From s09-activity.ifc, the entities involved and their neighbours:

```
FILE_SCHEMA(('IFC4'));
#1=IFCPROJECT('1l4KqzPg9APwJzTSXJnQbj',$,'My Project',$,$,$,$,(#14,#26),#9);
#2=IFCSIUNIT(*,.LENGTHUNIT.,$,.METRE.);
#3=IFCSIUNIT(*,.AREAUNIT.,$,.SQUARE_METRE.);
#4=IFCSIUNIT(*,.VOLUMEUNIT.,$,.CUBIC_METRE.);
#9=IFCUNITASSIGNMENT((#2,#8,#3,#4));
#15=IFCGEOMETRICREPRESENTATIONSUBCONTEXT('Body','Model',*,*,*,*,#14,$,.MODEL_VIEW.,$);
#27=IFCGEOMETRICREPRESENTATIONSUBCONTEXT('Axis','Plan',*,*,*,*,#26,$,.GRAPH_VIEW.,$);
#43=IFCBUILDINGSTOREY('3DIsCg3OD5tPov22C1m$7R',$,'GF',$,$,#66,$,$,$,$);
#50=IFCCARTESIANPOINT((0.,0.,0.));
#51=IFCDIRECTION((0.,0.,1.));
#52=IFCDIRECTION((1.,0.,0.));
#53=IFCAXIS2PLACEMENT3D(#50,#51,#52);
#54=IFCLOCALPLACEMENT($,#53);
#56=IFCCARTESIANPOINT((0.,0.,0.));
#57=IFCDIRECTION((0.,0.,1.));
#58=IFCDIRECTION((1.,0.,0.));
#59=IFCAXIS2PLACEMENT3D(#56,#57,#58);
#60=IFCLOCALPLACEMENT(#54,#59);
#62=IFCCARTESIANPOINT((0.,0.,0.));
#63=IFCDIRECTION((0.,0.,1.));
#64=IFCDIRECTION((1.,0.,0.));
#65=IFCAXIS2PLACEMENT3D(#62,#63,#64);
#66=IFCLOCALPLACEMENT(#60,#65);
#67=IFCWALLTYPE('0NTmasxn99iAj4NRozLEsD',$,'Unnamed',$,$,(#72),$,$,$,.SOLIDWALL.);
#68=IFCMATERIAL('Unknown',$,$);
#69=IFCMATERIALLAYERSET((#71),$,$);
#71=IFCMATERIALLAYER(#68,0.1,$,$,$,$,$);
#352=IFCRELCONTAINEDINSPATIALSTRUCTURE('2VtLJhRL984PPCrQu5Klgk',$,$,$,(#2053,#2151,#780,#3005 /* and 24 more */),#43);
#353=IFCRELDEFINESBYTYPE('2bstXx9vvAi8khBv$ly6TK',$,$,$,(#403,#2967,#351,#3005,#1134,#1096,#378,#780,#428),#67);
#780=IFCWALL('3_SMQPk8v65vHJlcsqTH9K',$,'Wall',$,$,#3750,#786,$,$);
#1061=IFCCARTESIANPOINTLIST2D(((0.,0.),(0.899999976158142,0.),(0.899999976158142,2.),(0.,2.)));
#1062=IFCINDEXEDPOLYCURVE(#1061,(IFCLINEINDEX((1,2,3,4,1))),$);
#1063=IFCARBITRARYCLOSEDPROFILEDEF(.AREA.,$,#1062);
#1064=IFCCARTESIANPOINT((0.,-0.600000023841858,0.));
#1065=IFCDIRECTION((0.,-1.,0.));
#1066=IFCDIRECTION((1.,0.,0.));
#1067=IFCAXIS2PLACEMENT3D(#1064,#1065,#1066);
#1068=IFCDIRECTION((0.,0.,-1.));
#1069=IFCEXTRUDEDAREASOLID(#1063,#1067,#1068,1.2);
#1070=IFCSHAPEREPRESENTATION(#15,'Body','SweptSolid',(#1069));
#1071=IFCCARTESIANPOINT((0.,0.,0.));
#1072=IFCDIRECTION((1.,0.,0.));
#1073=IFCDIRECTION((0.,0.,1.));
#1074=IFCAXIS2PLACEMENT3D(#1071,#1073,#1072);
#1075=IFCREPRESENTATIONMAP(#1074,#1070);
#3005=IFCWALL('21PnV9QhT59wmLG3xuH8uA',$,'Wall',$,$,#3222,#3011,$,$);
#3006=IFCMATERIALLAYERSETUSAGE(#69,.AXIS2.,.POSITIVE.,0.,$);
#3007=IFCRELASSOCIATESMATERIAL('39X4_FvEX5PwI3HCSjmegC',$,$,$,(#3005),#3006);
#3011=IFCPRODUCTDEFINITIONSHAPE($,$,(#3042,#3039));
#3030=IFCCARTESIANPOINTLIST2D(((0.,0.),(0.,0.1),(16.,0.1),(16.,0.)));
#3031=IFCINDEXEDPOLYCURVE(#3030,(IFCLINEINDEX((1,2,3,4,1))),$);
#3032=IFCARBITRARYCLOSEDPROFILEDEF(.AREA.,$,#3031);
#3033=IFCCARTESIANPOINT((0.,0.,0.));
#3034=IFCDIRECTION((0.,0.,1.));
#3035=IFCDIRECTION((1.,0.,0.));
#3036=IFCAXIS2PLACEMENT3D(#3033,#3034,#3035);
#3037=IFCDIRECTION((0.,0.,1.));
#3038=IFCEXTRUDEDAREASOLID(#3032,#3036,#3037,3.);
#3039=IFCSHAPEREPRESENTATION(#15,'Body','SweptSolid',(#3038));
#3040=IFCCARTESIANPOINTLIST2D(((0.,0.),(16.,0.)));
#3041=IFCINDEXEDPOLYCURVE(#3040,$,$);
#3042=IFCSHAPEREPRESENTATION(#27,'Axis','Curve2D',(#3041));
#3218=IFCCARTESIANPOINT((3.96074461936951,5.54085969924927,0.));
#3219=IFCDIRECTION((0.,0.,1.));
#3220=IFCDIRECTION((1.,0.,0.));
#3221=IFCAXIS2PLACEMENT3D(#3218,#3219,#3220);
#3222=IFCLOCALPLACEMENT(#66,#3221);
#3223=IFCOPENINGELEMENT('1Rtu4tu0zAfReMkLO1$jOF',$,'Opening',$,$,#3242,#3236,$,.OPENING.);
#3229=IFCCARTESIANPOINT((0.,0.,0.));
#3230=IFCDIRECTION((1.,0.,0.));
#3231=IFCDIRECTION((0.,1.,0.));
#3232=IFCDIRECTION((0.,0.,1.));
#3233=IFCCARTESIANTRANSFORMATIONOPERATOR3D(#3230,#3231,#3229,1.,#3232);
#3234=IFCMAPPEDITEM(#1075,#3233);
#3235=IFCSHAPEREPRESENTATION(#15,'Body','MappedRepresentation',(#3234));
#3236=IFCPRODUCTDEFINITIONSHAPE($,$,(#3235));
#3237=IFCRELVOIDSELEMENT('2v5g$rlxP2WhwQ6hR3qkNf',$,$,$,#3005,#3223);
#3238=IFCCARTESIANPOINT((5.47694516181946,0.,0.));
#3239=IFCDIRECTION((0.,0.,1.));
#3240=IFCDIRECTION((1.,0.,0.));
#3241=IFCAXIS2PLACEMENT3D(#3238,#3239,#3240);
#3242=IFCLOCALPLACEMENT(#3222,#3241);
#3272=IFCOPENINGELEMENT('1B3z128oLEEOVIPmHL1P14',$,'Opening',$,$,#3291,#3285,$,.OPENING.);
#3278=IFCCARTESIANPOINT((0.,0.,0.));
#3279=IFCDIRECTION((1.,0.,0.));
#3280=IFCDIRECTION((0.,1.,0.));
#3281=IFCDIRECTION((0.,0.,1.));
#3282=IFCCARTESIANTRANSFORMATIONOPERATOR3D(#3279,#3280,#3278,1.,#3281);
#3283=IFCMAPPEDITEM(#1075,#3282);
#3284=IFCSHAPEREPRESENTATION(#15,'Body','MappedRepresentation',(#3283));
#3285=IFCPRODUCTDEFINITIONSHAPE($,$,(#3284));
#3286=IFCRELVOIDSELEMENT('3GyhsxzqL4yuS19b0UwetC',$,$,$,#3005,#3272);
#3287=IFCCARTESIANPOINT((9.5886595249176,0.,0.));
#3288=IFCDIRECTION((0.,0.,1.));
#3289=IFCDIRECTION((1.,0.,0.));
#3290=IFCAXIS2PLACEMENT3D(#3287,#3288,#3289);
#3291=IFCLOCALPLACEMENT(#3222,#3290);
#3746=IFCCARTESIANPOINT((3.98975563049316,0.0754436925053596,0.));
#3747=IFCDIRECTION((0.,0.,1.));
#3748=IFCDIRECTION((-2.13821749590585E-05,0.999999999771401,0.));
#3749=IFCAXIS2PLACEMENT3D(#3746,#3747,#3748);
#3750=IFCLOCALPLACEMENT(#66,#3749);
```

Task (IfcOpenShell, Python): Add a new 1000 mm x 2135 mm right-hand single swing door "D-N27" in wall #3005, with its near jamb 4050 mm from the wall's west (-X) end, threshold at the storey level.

```python
import numpy as np
import ifcopenshell
import ifcopenshell.api.feature
import ifcopenshell.api.geometry
import ifcopenshell.api.root
import ifcopenshell.api.spatial
import ifcopenshell.geom
import ifcopenshell.util.element
import ifcopenshell.util.placement
import ifcopenshell.util.representation
import ifcopenshell.util.shape
import ifcopenshell.util.unit

model = ifcopenshell.open("s09-activity.ifc")
unit_scale = ifcopenshell.util.unit.calculate_unit_scale(model)
settings = ifcopenshell.geom.settings()


def volume(element):
    """Net volume in cubic metres, openings subtracted."""
    shape = ifcopenshell.geom.create_shape(settings, element)
    return ifcopenshell.util.shape.get_volume(shape.geometry)


wall = model.by_guid("21PnV9QhT59wmLG3xuH8uA")
storey = ifcopenshell.util.element.get_container(wall, ifc_class="IfcBuildingStorey")
context = ifcopenshell.util.representation.get_context(model, "Model", "Body", "MODEL_VIEW")
before = volume(wall)

width, height, from_end, sill = 1, 2.135, 4.05, 0.0  # metres

# The wall runs along its own X axis, and the end named is its -X end.
wall_shape = ifcopenshell.geom.create_shape(settings, wall)
x, y, z = ifcopenshell.util.shape.get_vertices(wall_shape.geometry).T
start = x.min() + from_end
face, thickness = float(y.min()), float(y.max() - y.min())
wall_matrix = ifcopenshell.util.placement.get_local_placement(wall.ObjectPlacement)
level = ifcopenshell.util.placement.get_local_placement(storey.ObjectPlacement)[2, 3]


def in_wall(x, y):
    """Placement at x, y metres in the wall's axes, at sill height."""
    matrix = wall_matrix.copy()
    matrix[:, 3] = wall_matrix @ np.array([x / unit_scale, y / unit_scale, 0.0, 1.0])
    matrix[2, 3] = level + sill / unit_scale
    return matrix


# Opening: a box that overshoots both wall faces by 50 mm.
opening = ifcopenshell.api.root.create_entity(model, ifc_class="IfcOpeningElement", predefined_type="OPENING")
box = ifcopenshell.api.geometry.add_wall_representation(
    model, context=context, length=width, height=height, thickness=thickness + 0.1
)
ifcopenshell.api.geometry.assign_representation(model, product=opening, representation=box)
ifcopenshell.api.geometry.edit_object_placement(model, product=opening, matrix=in_wall(start, face - 0.05), is_si=False)
ifcopenshell.api.feature.add_feature(model, feature=opening, element=wall)

door = ifcopenshell.api.root.create_entity(model, ifc_class="IfcDoor", name="D-N27", predefined_type="DOOR")
door.OverallWidth, door.OverallHeight = width / unit_scale, height / unit_scale
door.OperationType = "SINGLE_SWING_RIGHT"
body = ifcopenshell.api.geometry.add_door_representation(
    model,
    context=context,
    overall_width=door.OverallWidth,
    overall_height=door.OverallHeight,
    operation_type="SINGLE_SWING_RIGHT",
    lining_properties={"LiningDepth": thickness / unit_scale, "ThresholdDepth": thickness / unit_scale},
)
ifcopenshell.api.geometry.assign_representation(model, product=door, representation=body)
ifcopenshell.api.spatial.assign_container(model, products=[door], relating_structure=storey)
ifcopenshell.api.feature.add_filling(model, opening=opening, element=door)

# The lining spans the wall, so the door starts at the wall face.
ifcopenshell.api.geometry.edit_object_placement(model, product=door, matrix=in_wall(start, face), is_si=False)

after = volume(wall)

print(f"wall volume {before:.3f} -> {after:.3f} m3")

model.write("s09-activity_updated.ifc")
```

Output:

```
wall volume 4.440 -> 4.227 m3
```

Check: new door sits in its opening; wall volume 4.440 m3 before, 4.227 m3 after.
